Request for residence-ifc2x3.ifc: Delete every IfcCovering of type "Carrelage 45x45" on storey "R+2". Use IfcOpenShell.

First a look at what the model holds.

```python
import ifcopenshell
import ifcopenshell.util.element

model = ifcopenshell.open("residence-ifc2x3.ifc")
print(model.schema)
storey = next(s for s in model.by_type("IfcBuildingStorey") if s.Name == "R+2")
coverings = [e for e in ifcopenshell.util.element.get_decomposition(storey) if e.is_a("IfcCovering")]
seen = {}
for e in coverings:
    element_type = ifcopenshell.util.element.get_type(e)
    name = element_type.Name if element_type not in (None, e) else None
    seen[name] = seen.get(name, 0) + 1
for name, count in sorted(seen.items(), key=str):
    print(count, "x", name)
```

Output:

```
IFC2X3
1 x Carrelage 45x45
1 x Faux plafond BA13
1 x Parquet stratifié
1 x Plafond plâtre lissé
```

```python
import ifcopenshell
import ifcopenshell.api.root
import ifcopenshell.util.element

model = ifcopenshell.open("residence-ifc2x3.ifc")

storey = next(s for s in model.by_type("IfcBuildingStorey") if s.Name == "R+2")
coverings = [e for e in ifcopenshell.util.element.get_decomposition(storey) if e.is_a("IfcCovering")]
targets = [e for e in coverings if (t := ifcopenshell.util.element.get_type(e)) not in (None, e) and t.Name == "Carrelage 45x45"]

for e in targets:
    ifcopenshell.api.root.remove_product(model, product=e)
print(len(targets), "removed")

model.write("residence-ifc2x3_updated.ifc")
```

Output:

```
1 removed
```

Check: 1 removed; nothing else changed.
